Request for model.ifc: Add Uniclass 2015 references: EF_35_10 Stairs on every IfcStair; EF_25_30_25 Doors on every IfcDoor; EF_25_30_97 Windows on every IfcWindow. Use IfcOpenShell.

First a look at what the model holds.

```python
import ifcopenshell

model = ifcopenshell.open("model.ifc")
print(model.schema)
print("classifications:", [c.Name for c in model.by_type("IfcClassification")])
for ifc_class in ("IfcDoor", "IfcRoof", "IfcStair", "IfcWall", "IfcWindow"):
    print(ifc_class, len(model.by_type(ifc_class)))
```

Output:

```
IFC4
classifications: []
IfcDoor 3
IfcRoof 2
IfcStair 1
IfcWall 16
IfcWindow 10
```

```python
import ifcopenshell
import ifcopenshell.api.classification

model = ifcopenshell.open("model.ifc")

system = ifcopenshell.api.classification.add_classification(model, classification="Uniclass 2015")

codes = {
    "IfcStair": ("EF_35_10", "Stairs"),
    "IfcDoor": ("EF_25_30_25", "Doors"),
    "IfcWindow": ("EF_25_30_97", "Windows"),
}
for ifc_class, (code, name) in codes.items():
    products = model.by_type(ifc_class)
    ifcopenshell.api.classification.add_reference(
        model, products=products, classification=system, identification=code, name=name
    )
    print(code, len(products))

model.write("model_edited.ifc")
```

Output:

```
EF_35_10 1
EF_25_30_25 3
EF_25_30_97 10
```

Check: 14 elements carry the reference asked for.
